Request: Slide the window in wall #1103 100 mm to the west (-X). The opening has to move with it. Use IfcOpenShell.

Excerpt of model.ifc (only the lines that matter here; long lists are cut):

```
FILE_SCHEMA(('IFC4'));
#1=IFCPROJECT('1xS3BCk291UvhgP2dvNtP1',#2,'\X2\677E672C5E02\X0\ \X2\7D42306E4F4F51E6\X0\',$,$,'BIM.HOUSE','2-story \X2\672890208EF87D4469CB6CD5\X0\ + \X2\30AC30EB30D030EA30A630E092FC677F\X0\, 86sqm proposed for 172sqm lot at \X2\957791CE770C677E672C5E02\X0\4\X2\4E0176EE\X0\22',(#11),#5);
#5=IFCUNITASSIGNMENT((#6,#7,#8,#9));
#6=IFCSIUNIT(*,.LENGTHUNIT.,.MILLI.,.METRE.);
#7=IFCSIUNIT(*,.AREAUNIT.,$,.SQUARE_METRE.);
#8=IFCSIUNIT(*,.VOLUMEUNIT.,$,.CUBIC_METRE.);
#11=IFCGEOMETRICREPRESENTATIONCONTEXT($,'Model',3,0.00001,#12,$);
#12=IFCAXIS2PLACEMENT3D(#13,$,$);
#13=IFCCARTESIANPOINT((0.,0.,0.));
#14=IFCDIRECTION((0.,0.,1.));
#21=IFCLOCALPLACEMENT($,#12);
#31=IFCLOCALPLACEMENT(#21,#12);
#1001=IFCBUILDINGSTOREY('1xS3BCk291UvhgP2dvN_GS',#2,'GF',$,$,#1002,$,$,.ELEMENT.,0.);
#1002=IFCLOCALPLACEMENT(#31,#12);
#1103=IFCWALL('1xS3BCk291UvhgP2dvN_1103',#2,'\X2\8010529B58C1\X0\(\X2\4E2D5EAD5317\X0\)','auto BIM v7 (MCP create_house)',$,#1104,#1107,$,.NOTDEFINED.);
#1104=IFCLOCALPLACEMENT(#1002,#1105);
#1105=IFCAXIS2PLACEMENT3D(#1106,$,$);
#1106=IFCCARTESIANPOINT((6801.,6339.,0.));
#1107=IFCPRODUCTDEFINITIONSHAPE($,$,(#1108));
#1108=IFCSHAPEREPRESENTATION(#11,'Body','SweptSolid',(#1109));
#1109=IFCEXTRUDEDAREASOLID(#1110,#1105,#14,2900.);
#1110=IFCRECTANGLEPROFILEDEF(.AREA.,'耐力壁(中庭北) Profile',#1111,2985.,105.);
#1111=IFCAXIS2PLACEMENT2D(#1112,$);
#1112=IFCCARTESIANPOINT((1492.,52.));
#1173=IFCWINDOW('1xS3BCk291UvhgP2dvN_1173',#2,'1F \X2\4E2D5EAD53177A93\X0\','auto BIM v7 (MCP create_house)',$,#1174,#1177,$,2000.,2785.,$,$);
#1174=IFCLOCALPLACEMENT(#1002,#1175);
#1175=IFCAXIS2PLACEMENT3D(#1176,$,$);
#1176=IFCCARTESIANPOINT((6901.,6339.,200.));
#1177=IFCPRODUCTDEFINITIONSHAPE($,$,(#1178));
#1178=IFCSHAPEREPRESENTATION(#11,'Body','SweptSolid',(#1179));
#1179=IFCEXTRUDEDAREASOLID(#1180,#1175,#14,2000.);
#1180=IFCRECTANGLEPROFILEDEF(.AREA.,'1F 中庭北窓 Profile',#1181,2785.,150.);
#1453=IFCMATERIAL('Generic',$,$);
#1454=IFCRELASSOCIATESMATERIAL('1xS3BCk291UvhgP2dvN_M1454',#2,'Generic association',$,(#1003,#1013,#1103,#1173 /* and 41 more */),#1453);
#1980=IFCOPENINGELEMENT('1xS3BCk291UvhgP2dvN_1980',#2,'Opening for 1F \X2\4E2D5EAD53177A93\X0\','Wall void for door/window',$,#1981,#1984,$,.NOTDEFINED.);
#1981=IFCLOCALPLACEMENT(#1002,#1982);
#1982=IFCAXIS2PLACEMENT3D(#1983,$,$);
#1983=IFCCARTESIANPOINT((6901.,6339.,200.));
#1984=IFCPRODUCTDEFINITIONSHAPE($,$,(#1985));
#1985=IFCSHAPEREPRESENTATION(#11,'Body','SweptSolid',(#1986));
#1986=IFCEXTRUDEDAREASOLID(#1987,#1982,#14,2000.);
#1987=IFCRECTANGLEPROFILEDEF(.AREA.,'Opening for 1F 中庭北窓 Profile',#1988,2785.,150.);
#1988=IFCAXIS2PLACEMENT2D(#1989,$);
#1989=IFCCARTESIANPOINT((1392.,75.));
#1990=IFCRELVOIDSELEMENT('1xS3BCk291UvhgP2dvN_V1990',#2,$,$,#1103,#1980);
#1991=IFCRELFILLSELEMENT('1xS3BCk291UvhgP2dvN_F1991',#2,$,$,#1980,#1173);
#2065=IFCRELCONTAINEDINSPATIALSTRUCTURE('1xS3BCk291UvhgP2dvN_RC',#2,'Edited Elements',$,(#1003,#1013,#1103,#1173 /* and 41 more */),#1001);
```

```python
import ifcopenshell
import ifcopenshell.api.geometry
import ifcopenshell.util.placement

model = ifcopenshell.open("model.ifc")

window = model.by_guid("1xS3BCk291UvhgP2dvN_1173")
opening = window.FillsVoids[0].RelatingOpeningElement
wall = opening.VoidsElements[0].RelatingBuildingElement

wall_matrix = ifcopenshell.util.placement.get_local_placement(wall.ObjectPlacement)
shift = wall_matrix[:3, 0] * -100.0
before = ifcopenshell.util.placement.get_local_placement(window.ObjectPlacement)[:3, 3].copy()

# The window is not placed relative to its opening, so move both.
for product in (opening, window):
    matrix = ifcopenshell.util.placement.get_local_placement(product.ObjectPlacement)
    matrix[:3, 3] += shift
    ifcopenshell.api.geometry.edit_object_placement(model, product=product, matrix=matrix, is_si=False)

after = ifcopenshell.util.placement.get_local_placement(window.ObjectPlacement)[:3, 3]
print("window moved by", (after - before).round(3) + 0.0)

model.write("model_v2.ifc")
```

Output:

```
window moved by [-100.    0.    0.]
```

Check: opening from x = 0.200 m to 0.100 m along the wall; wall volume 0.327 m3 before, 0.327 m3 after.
